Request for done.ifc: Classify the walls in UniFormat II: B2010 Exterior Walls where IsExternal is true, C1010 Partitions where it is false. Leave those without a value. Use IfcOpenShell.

First a look at what the model holds.

```python
import ifcopenshell
import ifcopenshell.util.element

model = ifcopenshell.open("done.ifc")
print(model.schema)
print("classifications:", [c.Name for c in model.by_type("IfcClassification")])
values = [ifcopenshell.util.element.get_pset(e, "Pset_WallCommon", "IsExternal") for e in model.by_type("IfcWall")]
for value in (True, False, None):
    print("IsExternal", value, values.count(value))
```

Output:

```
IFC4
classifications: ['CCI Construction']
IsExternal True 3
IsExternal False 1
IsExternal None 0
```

```python
import ifcopenshell
import ifcopenshell.api.classification
import ifcopenshell.util.element

model = ifcopenshell.open("done.ifc")

system = ifcopenshell.api.classification.add_classification(model, classification="UniFormat II")

walls = model.by_type("IfcWall")
external = {e: ifcopenshell.util.element.get_pset(e, "Pset_WallCommon", "IsExternal") for e in walls}
for flag, code, name in ((True, "B2010", "Exterior Walls"), (False, "C1010", "Partitions")):
    products = [e for e in walls if external[e] is flag]
    ifcopenshell.api.classification.add_reference(
        model, products=products, classification=system, identification=code, name=name
    )
    print(code, len(products))

model.write("done-out.ifc")
```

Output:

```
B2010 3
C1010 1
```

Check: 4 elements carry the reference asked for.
